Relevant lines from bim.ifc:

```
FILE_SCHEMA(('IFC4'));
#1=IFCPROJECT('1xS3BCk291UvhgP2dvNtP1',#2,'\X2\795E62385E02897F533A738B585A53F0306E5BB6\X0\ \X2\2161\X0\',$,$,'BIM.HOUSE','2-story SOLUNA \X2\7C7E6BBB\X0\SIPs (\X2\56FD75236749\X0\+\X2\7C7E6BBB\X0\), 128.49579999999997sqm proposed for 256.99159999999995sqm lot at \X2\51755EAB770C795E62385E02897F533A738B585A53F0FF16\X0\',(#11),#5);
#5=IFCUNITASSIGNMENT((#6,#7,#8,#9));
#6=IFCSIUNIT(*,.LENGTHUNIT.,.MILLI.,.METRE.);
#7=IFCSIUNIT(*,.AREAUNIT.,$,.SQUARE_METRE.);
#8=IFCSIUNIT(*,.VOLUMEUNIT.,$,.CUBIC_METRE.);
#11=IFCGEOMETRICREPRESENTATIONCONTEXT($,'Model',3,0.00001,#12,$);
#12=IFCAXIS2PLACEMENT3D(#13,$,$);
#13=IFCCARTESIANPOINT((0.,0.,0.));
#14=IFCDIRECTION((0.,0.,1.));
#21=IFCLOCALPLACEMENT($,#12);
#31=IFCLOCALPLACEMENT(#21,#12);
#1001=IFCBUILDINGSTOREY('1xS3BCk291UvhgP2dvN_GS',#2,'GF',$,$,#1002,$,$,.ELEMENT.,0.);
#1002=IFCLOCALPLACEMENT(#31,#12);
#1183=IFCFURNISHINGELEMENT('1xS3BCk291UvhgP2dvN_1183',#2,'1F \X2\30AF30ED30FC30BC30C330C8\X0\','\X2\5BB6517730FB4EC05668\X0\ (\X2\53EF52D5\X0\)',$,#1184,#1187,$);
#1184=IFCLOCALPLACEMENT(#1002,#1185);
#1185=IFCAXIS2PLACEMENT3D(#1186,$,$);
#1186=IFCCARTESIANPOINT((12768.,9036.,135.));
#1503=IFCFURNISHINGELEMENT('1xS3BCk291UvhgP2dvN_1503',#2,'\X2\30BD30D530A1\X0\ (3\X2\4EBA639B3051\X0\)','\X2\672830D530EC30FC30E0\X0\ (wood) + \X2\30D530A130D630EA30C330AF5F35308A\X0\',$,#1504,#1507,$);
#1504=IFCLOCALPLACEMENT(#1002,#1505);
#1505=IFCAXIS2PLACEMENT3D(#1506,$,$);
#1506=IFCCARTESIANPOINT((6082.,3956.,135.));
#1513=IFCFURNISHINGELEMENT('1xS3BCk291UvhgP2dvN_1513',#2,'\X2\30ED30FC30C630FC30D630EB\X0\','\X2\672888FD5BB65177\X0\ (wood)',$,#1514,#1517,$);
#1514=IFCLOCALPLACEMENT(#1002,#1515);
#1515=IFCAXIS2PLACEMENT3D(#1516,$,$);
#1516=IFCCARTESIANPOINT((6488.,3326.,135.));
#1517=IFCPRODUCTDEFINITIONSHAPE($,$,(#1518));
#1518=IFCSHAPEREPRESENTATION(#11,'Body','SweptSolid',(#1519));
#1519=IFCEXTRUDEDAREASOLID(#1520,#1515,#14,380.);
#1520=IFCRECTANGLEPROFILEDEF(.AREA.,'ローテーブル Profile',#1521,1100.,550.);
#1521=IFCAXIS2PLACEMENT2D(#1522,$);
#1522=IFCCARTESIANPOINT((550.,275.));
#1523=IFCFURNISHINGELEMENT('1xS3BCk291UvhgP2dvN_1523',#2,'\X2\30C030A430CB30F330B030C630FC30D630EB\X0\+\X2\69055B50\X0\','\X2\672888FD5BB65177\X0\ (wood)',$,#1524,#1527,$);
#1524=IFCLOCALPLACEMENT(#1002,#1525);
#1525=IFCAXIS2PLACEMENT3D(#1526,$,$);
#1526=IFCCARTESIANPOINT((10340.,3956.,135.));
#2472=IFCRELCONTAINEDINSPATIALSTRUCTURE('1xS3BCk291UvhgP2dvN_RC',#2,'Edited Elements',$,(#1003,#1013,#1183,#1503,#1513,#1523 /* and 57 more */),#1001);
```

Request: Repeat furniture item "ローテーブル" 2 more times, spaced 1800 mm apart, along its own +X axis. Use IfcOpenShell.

```python
import ifcopenshell
import ifcopenshell.api.geometry
import ifcopenshell.api.root
import ifcopenshell.util.element
import ifcopenshell.util.placement

model = ifcopenshell.open("bim.ifc")


def reuse_history(source, copy):
    """copy_class also copies each property set's owner history, people and application; keep the originals."""
    for rel in copy.IsDefinedBy:
        if rel.is_a("IfcRelDefinesByProperties") and (history := rel.RelatingPropertyDefinition.OwnerHistory):
            rel.RelatingPropertyDefinition.OwnerHistory = source.OwnerHistory
            ifcopenshell.util.element.remove_deep2(model, history)


source = model.by_guid("1xS3BCk291UvhgP2dvN_1513")
base = ifcopenshell.util.placement.get_local_placement(source.ObjectPlacement)
step = base[:3, 0] * 1800.0

for i in range(1, 3):
    copy = ifcopenshell.api.root.copy_class(model, product=source)
    copy.Representation = ifcopenshell.util.element.copy_deep(
        model, source.Representation, exclude=["IfcGeometricRepresentationContext", "IfcRepresentationMap"]
    )
    reuse_history(source, copy)
    matrix = base.copy()
    matrix[:3, 3] += i * step
    print("added at", matrix[:3, 3].round(3) + 0.0)
    ifcopenshell.api.geometry.edit_object_placement(model, product=copy, matrix=matrix, is_si=False)

model.write("bim_rev.ifc")
```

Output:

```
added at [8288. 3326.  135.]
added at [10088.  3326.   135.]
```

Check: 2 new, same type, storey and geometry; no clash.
